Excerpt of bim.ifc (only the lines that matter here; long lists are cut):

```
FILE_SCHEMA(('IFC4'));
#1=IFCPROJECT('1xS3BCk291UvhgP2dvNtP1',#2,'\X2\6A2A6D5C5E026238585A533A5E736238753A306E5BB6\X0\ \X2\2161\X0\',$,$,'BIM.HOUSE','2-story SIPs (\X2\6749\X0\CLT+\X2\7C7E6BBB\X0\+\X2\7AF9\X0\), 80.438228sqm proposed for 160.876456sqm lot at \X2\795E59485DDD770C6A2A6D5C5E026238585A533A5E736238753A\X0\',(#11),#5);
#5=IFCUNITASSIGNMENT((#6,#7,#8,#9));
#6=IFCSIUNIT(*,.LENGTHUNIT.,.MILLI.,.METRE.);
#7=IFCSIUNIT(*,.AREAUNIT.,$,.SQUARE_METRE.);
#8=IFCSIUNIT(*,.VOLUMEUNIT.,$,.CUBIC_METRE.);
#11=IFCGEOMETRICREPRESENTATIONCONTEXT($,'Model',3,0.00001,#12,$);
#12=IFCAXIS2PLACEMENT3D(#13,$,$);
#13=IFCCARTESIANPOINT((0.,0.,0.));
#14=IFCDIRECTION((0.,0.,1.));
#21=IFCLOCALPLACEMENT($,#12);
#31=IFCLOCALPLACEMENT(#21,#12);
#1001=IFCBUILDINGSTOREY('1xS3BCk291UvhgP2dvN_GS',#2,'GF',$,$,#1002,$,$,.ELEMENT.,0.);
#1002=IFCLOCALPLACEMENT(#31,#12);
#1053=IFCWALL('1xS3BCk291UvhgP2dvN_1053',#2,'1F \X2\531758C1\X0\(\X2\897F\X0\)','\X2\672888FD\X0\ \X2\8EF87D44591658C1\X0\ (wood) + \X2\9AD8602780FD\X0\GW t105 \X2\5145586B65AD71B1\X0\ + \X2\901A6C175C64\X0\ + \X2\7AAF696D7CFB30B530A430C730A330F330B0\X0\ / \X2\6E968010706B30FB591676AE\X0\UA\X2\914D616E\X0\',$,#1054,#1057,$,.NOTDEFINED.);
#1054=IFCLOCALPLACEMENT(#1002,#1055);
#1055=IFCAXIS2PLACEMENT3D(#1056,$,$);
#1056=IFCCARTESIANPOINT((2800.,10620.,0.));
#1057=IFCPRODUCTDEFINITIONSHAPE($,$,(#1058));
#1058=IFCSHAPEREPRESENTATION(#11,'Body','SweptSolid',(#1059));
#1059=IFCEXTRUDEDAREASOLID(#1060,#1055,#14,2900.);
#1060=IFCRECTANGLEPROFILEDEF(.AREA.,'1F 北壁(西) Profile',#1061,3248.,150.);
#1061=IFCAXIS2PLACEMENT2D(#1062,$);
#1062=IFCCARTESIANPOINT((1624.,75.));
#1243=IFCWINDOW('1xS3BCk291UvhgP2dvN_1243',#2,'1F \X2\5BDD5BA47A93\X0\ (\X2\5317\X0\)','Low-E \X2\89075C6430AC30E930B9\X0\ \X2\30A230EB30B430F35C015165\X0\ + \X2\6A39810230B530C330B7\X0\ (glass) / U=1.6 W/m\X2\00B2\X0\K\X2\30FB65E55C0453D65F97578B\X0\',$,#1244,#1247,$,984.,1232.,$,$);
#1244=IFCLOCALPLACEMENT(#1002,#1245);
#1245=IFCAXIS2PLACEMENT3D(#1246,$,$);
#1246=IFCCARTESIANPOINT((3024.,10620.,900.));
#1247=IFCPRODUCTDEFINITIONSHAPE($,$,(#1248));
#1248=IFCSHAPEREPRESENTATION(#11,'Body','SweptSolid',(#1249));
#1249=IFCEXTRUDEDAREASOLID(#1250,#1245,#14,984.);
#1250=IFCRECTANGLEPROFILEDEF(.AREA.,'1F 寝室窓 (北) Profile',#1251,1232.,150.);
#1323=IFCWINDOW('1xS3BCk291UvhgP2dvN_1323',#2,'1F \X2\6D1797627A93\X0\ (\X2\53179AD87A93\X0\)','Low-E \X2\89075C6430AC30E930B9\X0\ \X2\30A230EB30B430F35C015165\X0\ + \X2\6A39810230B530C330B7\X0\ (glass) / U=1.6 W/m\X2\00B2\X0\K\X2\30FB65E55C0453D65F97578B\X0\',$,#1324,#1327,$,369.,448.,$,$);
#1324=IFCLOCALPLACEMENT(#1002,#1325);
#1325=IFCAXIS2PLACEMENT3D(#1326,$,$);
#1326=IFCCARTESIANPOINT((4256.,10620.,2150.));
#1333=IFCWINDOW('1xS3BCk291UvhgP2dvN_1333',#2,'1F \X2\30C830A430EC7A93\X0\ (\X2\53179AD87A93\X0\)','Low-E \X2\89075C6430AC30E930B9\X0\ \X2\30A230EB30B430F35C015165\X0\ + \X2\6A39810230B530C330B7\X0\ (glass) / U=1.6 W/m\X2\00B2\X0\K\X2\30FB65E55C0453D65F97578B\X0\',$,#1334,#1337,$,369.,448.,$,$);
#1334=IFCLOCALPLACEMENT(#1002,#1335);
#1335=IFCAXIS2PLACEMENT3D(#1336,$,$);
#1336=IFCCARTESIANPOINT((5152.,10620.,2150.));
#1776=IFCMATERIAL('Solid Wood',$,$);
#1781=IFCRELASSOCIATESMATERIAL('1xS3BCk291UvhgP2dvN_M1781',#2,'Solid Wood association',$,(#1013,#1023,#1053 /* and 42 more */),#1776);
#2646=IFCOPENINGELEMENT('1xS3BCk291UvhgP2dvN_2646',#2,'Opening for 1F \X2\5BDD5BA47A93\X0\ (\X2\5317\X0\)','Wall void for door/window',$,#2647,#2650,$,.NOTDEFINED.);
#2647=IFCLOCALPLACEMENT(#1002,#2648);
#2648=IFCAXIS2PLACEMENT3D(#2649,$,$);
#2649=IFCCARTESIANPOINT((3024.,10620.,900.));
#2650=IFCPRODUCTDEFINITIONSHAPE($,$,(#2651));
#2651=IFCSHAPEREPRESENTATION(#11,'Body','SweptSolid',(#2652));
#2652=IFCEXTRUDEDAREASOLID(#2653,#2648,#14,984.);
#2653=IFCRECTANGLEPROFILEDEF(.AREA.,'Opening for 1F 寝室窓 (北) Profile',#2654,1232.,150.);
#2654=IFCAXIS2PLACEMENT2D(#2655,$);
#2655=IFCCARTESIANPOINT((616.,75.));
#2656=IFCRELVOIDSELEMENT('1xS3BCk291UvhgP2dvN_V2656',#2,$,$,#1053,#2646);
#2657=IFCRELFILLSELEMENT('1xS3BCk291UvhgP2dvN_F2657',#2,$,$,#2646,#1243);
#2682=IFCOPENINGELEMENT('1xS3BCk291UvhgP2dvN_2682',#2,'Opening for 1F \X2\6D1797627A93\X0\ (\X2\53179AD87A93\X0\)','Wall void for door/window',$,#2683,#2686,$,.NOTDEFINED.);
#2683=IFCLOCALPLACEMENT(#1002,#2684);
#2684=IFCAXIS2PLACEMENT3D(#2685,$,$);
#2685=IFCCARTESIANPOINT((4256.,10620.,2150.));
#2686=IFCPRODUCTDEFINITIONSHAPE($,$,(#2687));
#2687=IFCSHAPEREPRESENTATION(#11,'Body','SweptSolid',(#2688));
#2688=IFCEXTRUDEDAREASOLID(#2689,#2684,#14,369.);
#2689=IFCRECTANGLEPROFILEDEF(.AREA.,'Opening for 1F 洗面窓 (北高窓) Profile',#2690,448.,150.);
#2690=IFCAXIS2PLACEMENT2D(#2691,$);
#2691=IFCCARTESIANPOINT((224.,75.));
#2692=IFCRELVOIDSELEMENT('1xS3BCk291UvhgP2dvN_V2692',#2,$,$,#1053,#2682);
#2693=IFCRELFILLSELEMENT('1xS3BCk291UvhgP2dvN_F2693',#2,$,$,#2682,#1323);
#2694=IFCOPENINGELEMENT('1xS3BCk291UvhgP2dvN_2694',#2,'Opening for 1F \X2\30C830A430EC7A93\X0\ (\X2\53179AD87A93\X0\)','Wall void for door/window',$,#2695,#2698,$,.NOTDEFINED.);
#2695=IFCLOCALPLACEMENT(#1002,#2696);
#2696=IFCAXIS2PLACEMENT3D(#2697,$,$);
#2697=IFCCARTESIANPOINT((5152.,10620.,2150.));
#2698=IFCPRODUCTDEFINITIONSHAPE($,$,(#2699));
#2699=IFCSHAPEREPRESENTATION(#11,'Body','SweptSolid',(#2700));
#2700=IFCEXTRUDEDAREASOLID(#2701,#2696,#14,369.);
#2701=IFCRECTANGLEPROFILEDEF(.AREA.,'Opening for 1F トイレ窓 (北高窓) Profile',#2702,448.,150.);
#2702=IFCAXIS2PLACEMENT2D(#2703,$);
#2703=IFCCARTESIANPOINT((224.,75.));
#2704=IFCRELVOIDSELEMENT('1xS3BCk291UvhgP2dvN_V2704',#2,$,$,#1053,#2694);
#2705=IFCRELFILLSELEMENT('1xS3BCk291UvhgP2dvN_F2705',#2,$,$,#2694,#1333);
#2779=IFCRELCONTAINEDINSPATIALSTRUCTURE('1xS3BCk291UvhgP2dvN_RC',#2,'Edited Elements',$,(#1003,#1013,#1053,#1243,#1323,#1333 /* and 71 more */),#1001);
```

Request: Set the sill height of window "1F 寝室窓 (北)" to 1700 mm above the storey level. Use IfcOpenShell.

```python
import numpy as np
import ifcopenshell
import ifcopenshell.api.geometry
import ifcopenshell.geom
import ifcopenshell.util.element
import ifcopenshell.util.placement
import ifcopenshell.util.shape
import ifcopenshell.util.unit

model = ifcopenshell.open("bim.ifc")
unit_scale = ifcopenshell.util.unit.calculate_unit_scale(model)

window = model.by_guid("1xS3BCk291UvhgP2dvN_1243")
opening = window.FillsVoids[0].RelatingOpeningElement
storey = ifcopenshell.util.element.get_container(window, ifc_class="IfcBuildingStorey")
level = ifcopenshell.util.placement.get_local_placement(storey.ObjectPlacement)[2, 3]

# The opening's origin need not be at the sill, so measure its lowest point.
shape = ifcopenshell.geom.create_shape(ifcopenshell.geom.settings(), opening)
bottom = ifcopenshell.util.shape.get_shape_bottom_elevation(shape, shape.geometry) / unit_scale
dz = level + 1.7 / unit_scale - bottom

shift = np.array([0.0, 0.0, dz])
# The window is not placed relative to its opening, so move both.
for product in (opening, window):
    matrix = ifcopenshell.util.placement.get_local_placement(product.ObjectPlacement)
    matrix[:3, 3] += shift
    ifcopenshell.api.geometry.edit_object_placement(model, product=product, matrix=matrix, is_si=False)

print(f"moved by {dz * unit_scale:+.3f} m")

model.write("bim-out.ifc")
```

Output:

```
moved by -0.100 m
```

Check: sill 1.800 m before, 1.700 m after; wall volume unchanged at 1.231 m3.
